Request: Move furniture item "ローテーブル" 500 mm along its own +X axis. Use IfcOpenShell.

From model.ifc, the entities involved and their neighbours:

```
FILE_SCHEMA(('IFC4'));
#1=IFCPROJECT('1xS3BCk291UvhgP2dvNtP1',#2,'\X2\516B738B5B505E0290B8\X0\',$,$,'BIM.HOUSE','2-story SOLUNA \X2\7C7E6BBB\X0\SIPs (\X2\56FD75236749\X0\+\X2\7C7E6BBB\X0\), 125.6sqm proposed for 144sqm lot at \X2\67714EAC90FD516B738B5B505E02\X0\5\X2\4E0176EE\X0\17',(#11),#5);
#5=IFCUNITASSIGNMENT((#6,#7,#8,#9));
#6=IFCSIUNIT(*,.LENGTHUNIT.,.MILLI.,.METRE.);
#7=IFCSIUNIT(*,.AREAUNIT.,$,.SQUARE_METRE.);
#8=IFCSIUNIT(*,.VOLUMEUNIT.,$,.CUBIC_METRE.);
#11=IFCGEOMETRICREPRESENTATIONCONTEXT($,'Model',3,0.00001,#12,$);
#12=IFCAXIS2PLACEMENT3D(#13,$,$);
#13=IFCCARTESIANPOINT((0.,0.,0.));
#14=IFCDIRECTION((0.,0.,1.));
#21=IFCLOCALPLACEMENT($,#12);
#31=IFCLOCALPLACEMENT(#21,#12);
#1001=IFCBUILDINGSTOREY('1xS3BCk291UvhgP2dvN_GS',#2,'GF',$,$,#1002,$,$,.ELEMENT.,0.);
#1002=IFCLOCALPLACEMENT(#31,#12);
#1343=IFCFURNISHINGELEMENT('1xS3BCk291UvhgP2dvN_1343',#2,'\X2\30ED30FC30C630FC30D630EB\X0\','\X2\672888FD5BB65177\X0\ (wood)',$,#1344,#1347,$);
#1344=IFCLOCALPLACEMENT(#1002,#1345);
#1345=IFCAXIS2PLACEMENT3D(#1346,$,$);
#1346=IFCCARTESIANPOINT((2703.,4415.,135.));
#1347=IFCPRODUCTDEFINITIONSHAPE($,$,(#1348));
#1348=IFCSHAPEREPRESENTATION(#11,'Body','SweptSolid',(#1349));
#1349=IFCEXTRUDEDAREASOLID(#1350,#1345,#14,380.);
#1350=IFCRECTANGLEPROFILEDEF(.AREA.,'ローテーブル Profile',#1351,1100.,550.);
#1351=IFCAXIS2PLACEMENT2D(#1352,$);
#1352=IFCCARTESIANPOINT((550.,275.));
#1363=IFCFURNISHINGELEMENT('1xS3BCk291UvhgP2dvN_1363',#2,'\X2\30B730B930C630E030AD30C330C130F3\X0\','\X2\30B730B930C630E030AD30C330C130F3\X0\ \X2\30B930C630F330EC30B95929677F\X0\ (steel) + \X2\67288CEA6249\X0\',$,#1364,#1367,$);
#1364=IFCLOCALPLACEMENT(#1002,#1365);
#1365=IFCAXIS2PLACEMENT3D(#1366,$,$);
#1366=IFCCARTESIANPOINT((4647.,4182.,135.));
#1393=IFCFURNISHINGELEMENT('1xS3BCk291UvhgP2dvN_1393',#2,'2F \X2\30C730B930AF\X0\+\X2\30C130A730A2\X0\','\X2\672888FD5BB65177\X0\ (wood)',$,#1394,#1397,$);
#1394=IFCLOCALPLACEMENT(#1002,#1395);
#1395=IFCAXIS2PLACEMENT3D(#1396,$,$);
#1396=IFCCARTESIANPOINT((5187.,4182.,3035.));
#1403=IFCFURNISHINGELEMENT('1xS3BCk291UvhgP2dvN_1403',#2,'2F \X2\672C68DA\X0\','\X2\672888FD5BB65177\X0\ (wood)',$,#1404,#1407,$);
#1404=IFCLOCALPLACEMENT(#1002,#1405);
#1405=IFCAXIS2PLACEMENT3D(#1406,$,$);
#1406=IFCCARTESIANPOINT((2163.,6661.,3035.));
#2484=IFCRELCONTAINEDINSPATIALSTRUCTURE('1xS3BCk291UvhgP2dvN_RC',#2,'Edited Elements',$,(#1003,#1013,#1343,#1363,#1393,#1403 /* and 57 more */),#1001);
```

```python
import ifcopenshell
import ifcopenshell.api.geometry
import ifcopenshell.util.placement
import ifcopenshell.util.unit

model = ifcopenshell.open("model.ifc")
unit_scale = ifcopenshell.util.unit.calculate_unit_scale(model)

item = model.by_id(1343)
matrix = ifcopenshell.util.placement.get_local_placement(item.ObjectPlacement)
matrix[:3, 3] += matrix[:3, 0] * 0.5 / unit_scale
ifcopenshell.api.geometry.edit_object_placement(model, product=item, matrix=matrix, is_si=False)

print(ifcopenshell.util.placement.get_local_placement(item.ObjectPlacement).round(3) + 0.0)

model.write("model_updated.ifc")
```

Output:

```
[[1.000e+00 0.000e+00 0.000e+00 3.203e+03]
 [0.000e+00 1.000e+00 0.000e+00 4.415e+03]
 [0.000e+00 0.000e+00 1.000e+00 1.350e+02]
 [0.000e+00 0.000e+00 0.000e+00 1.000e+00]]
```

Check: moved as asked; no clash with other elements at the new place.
